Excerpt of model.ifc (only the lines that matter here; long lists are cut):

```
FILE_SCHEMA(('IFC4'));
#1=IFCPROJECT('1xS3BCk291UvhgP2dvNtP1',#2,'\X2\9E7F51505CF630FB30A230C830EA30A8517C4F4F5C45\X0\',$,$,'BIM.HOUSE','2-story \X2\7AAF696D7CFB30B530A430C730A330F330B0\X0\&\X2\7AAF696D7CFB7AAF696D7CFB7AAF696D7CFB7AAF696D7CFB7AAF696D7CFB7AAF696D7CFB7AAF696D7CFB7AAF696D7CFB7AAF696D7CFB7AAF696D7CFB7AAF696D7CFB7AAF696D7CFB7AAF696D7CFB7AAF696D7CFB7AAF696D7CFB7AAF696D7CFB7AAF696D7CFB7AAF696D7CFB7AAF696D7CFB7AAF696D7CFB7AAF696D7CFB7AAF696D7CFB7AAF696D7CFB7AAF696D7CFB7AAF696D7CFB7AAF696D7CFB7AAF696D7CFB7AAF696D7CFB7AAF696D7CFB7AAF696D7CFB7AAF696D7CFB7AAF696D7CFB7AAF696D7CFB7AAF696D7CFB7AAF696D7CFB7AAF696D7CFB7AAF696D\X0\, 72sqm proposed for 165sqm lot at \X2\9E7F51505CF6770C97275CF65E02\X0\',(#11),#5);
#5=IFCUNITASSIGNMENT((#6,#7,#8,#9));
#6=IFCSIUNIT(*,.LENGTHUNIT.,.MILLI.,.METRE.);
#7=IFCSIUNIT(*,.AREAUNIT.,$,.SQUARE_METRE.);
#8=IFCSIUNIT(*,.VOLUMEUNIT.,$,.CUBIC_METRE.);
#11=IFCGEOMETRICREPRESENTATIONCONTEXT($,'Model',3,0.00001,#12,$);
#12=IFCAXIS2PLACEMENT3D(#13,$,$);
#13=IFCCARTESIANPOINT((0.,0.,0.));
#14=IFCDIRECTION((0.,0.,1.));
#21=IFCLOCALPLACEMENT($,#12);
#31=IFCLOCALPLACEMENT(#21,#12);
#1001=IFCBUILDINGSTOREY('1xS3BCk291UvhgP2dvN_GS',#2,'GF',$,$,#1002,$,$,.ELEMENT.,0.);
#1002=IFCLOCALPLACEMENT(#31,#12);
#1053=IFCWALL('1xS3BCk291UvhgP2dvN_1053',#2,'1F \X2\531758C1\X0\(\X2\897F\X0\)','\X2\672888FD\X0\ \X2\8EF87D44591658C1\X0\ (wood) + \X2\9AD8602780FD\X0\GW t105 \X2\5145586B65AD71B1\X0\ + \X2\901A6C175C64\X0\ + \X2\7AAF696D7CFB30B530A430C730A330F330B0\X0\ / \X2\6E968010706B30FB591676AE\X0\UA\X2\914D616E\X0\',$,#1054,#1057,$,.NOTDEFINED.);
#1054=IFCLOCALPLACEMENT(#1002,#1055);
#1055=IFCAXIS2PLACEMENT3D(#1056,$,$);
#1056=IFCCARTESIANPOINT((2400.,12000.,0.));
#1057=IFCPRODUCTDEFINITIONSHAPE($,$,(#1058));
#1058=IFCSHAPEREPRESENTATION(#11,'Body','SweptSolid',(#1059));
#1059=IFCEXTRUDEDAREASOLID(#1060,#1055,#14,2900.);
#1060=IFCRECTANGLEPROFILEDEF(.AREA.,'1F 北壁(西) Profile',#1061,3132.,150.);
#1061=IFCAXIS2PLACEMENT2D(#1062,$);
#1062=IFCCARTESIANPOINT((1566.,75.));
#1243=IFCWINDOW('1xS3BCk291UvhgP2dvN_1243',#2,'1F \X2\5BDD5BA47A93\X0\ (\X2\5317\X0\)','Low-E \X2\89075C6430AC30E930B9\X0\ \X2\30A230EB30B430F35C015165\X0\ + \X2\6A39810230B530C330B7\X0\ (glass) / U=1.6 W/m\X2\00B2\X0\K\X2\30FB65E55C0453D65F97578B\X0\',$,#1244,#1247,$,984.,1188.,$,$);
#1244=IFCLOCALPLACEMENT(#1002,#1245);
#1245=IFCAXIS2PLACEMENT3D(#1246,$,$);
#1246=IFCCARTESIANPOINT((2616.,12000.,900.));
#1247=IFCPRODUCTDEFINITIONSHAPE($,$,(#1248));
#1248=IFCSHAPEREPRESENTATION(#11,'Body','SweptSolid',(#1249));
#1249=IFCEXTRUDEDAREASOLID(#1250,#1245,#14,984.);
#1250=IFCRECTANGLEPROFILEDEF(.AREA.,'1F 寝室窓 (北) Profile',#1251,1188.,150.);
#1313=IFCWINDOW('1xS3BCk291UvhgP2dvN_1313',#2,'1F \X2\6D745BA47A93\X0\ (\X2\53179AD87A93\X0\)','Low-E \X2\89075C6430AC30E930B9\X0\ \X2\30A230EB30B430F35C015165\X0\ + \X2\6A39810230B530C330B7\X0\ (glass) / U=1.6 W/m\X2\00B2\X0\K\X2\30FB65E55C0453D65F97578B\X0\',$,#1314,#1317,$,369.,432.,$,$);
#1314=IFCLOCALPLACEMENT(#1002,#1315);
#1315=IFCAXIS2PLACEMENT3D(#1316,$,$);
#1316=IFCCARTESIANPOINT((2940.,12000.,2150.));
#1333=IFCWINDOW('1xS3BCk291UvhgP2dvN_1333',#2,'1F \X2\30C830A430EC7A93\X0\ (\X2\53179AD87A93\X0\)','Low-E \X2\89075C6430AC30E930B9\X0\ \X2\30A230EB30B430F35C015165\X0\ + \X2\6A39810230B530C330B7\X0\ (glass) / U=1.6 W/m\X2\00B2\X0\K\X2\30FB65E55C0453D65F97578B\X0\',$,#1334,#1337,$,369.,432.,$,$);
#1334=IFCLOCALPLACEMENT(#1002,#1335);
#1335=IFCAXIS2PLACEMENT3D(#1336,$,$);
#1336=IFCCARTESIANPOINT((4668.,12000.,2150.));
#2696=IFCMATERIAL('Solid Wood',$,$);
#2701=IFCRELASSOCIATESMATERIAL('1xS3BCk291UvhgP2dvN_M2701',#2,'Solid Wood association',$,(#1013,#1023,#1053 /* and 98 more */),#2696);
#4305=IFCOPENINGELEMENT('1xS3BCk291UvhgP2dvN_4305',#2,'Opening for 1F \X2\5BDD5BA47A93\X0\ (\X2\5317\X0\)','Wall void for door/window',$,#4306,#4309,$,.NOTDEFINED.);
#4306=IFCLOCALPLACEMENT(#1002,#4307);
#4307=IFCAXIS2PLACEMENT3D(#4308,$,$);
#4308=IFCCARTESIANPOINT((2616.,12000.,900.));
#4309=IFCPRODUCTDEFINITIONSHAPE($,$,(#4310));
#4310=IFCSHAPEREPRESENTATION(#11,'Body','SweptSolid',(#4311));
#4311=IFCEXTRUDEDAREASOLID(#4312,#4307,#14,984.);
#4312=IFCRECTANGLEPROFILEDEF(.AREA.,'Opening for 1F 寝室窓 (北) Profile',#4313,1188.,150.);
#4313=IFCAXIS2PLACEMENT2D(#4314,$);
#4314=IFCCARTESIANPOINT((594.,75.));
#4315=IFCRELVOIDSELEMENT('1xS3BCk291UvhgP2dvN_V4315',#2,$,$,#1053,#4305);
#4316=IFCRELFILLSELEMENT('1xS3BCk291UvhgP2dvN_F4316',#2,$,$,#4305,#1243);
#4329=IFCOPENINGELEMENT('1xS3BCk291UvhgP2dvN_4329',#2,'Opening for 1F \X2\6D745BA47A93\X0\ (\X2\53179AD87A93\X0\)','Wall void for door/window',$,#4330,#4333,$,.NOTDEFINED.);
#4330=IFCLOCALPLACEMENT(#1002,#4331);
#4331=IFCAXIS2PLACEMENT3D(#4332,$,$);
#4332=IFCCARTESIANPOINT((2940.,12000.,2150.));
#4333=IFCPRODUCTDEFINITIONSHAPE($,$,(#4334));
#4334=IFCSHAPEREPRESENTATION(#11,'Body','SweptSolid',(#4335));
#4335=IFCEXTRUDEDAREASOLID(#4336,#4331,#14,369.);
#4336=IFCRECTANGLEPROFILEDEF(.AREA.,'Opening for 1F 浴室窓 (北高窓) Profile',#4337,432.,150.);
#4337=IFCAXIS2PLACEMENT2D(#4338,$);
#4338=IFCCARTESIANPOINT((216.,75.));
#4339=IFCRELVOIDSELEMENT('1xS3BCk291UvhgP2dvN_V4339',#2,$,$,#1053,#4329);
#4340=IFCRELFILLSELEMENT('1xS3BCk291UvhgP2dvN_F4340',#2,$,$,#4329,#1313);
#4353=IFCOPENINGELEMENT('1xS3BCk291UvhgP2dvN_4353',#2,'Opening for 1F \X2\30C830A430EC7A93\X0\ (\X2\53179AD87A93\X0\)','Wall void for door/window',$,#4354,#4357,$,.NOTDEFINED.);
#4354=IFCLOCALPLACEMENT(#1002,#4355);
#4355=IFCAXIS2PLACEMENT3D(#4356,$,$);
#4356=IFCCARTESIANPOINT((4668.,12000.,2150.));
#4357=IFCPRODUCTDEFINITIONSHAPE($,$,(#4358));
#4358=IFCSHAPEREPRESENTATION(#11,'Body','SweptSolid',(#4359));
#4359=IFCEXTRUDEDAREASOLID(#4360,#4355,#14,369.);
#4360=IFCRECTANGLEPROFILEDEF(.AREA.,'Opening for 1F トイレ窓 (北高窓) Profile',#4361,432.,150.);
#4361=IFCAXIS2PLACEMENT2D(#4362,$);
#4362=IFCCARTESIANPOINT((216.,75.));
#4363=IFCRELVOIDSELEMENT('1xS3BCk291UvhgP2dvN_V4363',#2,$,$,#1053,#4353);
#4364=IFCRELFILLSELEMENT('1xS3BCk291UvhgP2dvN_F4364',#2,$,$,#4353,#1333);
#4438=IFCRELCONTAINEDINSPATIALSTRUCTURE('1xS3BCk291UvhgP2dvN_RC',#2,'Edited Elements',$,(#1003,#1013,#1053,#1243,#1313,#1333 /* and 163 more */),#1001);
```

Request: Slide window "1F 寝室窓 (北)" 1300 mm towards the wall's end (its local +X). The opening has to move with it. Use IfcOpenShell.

```python
import ifcopenshell
import ifcopenshell.api.geometry
import ifcopenshell.util.placement
import ifcopenshell.util.unit

model = ifcopenshell.open("model.ifc")
unit_scale = ifcopenshell.util.unit.calculate_unit_scale(model)

window = model.by_guid("1xS3BCk291UvhgP2dvN_1243")
opening = window.FillsVoids[0].RelatingOpeningElement
wall = opening.VoidsElements[0].RelatingBuildingElement

wall_matrix = ifcopenshell.util.placement.get_local_placement(wall.ObjectPlacement)
shift = wall_matrix[:3, 0] * 1.3 / unit_scale
before = ifcopenshell.util.placement.get_local_placement(window.ObjectPlacement)[:3, 3].copy()

# The window is not placed relative to its opening, so move both.
for product in (opening, window):
    matrix = ifcopenshell.util.placement.get_local_placement(product.ObjectPlacement)
    matrix[:3, 3] += shift
    ifcopenshell.api.geometry.edit_object_placement(model, product=product, matrix=matrix, is_si=False)

after = ifcopenshell.util.placement.get_local_placement(window.ObjectPlacement)[:3, 3]
print("window moved by", (after - before).round(3) + 0.0)

model.write("model_rev.ifc")
```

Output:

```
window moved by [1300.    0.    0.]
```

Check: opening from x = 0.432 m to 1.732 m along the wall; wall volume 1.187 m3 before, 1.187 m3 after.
